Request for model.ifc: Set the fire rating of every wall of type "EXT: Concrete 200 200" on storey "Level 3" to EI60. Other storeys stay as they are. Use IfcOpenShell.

First a look at what the model holds.

```python
import ifcopenshell
import ifcopenshell.util.element

model = ifcopenshell.open("model.ifc")
print(model.schema)
storey = next(s for s in model.by_type("IfcBuildingStorey") if s.Name == "Level 3")
walls = [e for e in ifcopenshell.util.element.get_decomposition(storey) if e.is_a("IfcWall")]
seen = {}
for e in walls:
    element_type = ifcopenshell.util.element.get_type(e)
    key = (element_type.Name if element_type != e and element_type else None, ifcopenshell.util.element.get_pset(e, "Pset_WallCommon", "FireRating"))
    seen[key] = seen.get(key, 0) + 1
for (name, value), count in sorted(seen.items(), key=str):
    print(count, "x", name, "|", value)
```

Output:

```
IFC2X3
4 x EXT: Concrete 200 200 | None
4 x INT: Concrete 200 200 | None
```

```python
import ifcopenshell
import ifcopenshell.api.pset
import ifcopenshell.util.element

model = ifcopenshell.open("model.ifc")

storey = next(s for s in model.by_type("IfcBuildingStorey") if s.Name == "Level 3")
walls = [e for e in ifcopenshell.util.element.get_decomposition(storey) if e.is_a("IfcWall")]

count = 0
for e in walls:
    element_type = ifcopenshell.util.element.get_type(e)
    if element_type in (None, e) or element_type.Name != "EXT: Concrete 200 200":
        continue
    # add_pset returns the element's existing set when there is one.
    pset = ifcopenshell.api.pset.add_pset(model, product=e, name="Pset_WallCommon")
    ifcopenshell.api.pset.edit_pset(model, pset=pset, properties={"FireRating": "EI60"})
    count += 1

print(count, "walls updated")

model.write("model-out.ifc")
```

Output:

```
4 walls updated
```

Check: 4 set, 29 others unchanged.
